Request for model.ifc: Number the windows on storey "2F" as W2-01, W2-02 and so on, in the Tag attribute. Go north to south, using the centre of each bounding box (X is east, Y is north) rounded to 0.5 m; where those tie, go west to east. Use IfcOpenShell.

First a look at what the model holds.

```python
import ifcopenshell
import ifcopenshell.util.element
import ifcopenshell.util.placement

model = ifcopenshell.open("model.ifc")
print(model.schema)
storey = next(s for s in model.by_type("IfcBuildingStorey") if s.Name == "2F")
windows = [e for e in ifcopenshell.util.element.get_decomposition(storey) if e.is_a("IfcWindow")]
for e in sorted(windows, key=lambda e: e.id()):
    origin = ifcopenshell.util.placement.get_local_placement(e.ObjectPlacement)[:3, 3]
    print(e.id(), e.Tag, e.Name, origin.round(2) + 0.0, sep=" | ")
```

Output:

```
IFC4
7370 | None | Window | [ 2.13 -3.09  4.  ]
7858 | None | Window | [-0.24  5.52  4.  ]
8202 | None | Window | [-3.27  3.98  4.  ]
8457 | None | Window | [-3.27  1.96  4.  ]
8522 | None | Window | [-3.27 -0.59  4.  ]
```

```python
import ifcopenshell
import ifcopenshell.geom
import ifcopenshell.util.element
import ifcopenshell.util.shape

model = ifcopenshell.open("model.ifc")
settings = ifcopenshell.geom.settings()
settings.set("use-world-coords", True)


def centre(element):
    shape = ifcopenshell.geom.create_shape(settings, element)
    return ifcopenshell.util.shape.get_bbox_centroid(shape.geometry)


storey = next(s for s in model.by_type("IfcBuildingStorey") if s.Name == "2F")
windows = [e for e in ifcopenshell.util.element.get_decomposition(storey) if e.is_a("IfcWindow")]

# Insertion points can sit at a corner or the storey origin, so sort by the geometry (in metres).
centres = {e: centre(e) for e in windows}
windows.sort(key=lambda e: (-round(centres[e][1] / 0.5), centres[e][0]))

for i, e in enumerate(windows, start=1):
    number = f"W2-{i:02d}"
    e.Tag = number
    print(e.id(), number)

model.write("model_edited.ifc")
```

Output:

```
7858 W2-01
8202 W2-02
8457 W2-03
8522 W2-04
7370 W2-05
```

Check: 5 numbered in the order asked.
